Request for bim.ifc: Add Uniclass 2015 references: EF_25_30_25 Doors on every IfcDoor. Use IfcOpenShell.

First a look at what the model holds.

```python
import ifcopenshell

model = ifcopenshell.open("bim.ifc")
print(model.schema)
print("classifications:", [c.Name for c in model.by_type("IfcClassification")])
for ifc_class in ("IfcDoor", "IfcRoof", "IfcStair", "IfcWall", "IfcWindow"):
    print(ifc_class, len(model.by_type(ifc_class)))
```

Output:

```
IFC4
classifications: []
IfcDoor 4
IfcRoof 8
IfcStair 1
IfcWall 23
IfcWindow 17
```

```python
import ifcopenshell
import ifcopenshell.api.classification

model = ifcopenshell.open("bim.ifc")

system = ifcopenshell.api.classification.add_classification(model, classification="Uniclass 2015")

codes = {
    "IfcDoor": ("EF_25_30_25", "Doors"),
}
for ifc_class, (code, name) in codes.items():
    products = model.by_type(ifc_class)
    ifcopenshell.api.classification.add_reference(
        model, products=products, classification=system, identification=code, name=name
    )
    print(code, len(products))

model.write("bim_updated.ifc")
```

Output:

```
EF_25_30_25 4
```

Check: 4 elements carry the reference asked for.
